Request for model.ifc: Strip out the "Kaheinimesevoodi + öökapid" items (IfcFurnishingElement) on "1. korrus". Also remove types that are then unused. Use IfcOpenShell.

First a look at what the model holds.

```python
import ifcopenshell
import ifcopenshell.util.element

model = ifcopenshell.open("model.ifc")
print(model.schema)
storey = next(s for s in model.by_type("IfcBuildingStorey") if s.Name == "1. korrus")
furniture = [e for e in ifcopenshell.util.element.get_decomposition(storey) if e.is_a("IfcFurnishingElement")]
seen = {}
for e in furniture:
    element_type = ifcopenshell.util.element.get_type(e)
    name = element_type.Name if element_type not in (None, e) else None
    seen[name] = seen.get(name, 0) + 1
for name, count in sorted(seen.items(), key=str):
    print(count, "x", name)
```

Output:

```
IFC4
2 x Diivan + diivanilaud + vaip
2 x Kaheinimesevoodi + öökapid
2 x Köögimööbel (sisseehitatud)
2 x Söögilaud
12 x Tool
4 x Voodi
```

```python
import ifcopenshell
import ifcopenshell.api.root
import ifcopenshell.util.element

model = ifcopenshell.open("model.ifc")

storey = next(s for s in model.by_type("IfcBuildingStorey") if s.Name == "1. korrus")
furniture = [e for e in ifcopenshell.util.element.get_decomposition(storey) if e.is_a("IfcFurnishingElement")]
targets = [e for e in furniture if (t := ifcopenshell.util.element.get_type(e)) not in (None, e) and t.Name == "Kaheinimesevoodi + öökapid"]
types = {ifcopenshell.util.element.get_type(e) for e in targets} - {None, *targets}

for e in targets:
    ifcopenshell.api.root.remove_product(model, product=e)
print(len(targets), "removed")

unused = [t for t in types if not ifcopenshell.util.element.get_types(t)]
for t in unused:
    ifcopenshell.api.root.remove_product(model, product=t)
print(len(unused), "unused types removed")

model.write("model-out.ifc")
```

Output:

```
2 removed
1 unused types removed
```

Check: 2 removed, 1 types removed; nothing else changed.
